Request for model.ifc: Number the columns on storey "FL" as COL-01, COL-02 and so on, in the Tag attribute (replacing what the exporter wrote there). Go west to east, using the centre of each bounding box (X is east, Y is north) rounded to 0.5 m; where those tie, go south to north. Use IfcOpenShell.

First a look at what the model holds.

```python
import ifcopenshell
import ifcopenshell.util.element
import ifcopenshell.util.placement

model = ifcopenshell.open("model.ifc")
print(model.schema)
storey = next(s for s in model.by_type("IfcBuildingStorey") if s.Name == "FL")
columns = [e for e in ifcopenshell.util.element.get_decomposition(storey) if e.is_a("IfcColumn")]
for e in sorted(columns, key=lambda e: e.id()):
    origin = ifcopenshell.util.placement.get_local_placement(e.ObjectPlacement)[:3, 3]
    print(e.id(), e.Tag, e.Name, origin.round(2) + 0.0, sep=" | ")
```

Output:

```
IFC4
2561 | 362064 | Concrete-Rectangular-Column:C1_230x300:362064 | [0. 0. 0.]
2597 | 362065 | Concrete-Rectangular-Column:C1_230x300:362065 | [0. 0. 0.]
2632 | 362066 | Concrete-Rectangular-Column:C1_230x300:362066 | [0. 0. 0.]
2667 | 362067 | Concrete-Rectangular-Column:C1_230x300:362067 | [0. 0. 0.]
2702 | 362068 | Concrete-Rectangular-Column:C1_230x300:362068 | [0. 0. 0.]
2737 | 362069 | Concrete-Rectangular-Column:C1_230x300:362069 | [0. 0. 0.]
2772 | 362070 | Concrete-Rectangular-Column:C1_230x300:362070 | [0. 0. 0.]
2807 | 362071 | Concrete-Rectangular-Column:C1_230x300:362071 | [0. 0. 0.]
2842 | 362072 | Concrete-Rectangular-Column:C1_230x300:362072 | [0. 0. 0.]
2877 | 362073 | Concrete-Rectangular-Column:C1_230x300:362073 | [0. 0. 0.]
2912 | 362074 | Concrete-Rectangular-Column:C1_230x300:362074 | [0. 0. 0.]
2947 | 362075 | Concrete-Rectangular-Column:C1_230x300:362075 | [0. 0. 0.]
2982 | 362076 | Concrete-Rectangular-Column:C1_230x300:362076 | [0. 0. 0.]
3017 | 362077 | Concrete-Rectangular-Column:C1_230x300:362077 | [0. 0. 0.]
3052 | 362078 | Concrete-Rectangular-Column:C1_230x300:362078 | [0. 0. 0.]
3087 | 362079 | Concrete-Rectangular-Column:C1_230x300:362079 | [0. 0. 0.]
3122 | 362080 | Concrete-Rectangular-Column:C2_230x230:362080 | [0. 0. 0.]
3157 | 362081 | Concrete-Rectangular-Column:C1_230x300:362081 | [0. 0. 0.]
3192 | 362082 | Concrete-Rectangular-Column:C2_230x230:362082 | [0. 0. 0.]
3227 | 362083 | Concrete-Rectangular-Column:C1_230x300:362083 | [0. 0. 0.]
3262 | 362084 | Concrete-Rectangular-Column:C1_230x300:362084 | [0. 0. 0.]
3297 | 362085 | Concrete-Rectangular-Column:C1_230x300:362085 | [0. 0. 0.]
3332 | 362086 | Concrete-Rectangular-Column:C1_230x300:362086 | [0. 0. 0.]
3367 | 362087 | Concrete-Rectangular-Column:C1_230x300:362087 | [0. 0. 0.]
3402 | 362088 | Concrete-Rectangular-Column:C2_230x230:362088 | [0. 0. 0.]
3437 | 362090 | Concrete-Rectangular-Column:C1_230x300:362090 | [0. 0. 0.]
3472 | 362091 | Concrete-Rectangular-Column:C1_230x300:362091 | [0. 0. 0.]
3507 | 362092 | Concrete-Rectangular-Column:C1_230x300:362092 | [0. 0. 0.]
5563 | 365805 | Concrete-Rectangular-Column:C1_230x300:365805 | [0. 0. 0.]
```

```python
import ifcopenshell
import ifcopenshell.geom
import ifcopenshell.util.element
import ifcopenshell.util.shape

model = ifcopenshell.open("model.ifc")
settings = ifcopenshell.geom.settings()
settings.set("use-world-coords", True)


def centre(element):
    shape = ifcopenshell.geom.create_shape(settings, element)
    return ifcopenshell.util.shape.get_bbox_centroid(shape.geometry)


storey = next(s for s in model.by_type("IfcBuildingStorey") if s.Name == "FL")
columns = [e for e in ifcopenshell.util.element.get_decomposition(storey) if e.is_a("IfcColumn")]

# Insertion points can sit at a corner or the storey origin, so sort by the geometry (in metres).
centres = {e: centre(e) for e in columns}
columns.sort(key=lambda e: (round(centres[e][0] / 0.5), centres[e][1]))

for i, e in enumerate(columns, start=1):
    number = f"COL-{i:02d}"
    e.Tag = number
    print(e.id(), number)

model.write("model-out.ifc")
```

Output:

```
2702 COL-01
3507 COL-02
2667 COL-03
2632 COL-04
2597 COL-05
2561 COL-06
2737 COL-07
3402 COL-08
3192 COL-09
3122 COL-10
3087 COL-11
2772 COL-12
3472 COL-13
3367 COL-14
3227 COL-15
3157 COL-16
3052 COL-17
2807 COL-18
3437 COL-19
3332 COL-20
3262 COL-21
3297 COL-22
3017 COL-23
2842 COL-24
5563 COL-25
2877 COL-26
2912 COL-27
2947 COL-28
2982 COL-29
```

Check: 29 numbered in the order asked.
